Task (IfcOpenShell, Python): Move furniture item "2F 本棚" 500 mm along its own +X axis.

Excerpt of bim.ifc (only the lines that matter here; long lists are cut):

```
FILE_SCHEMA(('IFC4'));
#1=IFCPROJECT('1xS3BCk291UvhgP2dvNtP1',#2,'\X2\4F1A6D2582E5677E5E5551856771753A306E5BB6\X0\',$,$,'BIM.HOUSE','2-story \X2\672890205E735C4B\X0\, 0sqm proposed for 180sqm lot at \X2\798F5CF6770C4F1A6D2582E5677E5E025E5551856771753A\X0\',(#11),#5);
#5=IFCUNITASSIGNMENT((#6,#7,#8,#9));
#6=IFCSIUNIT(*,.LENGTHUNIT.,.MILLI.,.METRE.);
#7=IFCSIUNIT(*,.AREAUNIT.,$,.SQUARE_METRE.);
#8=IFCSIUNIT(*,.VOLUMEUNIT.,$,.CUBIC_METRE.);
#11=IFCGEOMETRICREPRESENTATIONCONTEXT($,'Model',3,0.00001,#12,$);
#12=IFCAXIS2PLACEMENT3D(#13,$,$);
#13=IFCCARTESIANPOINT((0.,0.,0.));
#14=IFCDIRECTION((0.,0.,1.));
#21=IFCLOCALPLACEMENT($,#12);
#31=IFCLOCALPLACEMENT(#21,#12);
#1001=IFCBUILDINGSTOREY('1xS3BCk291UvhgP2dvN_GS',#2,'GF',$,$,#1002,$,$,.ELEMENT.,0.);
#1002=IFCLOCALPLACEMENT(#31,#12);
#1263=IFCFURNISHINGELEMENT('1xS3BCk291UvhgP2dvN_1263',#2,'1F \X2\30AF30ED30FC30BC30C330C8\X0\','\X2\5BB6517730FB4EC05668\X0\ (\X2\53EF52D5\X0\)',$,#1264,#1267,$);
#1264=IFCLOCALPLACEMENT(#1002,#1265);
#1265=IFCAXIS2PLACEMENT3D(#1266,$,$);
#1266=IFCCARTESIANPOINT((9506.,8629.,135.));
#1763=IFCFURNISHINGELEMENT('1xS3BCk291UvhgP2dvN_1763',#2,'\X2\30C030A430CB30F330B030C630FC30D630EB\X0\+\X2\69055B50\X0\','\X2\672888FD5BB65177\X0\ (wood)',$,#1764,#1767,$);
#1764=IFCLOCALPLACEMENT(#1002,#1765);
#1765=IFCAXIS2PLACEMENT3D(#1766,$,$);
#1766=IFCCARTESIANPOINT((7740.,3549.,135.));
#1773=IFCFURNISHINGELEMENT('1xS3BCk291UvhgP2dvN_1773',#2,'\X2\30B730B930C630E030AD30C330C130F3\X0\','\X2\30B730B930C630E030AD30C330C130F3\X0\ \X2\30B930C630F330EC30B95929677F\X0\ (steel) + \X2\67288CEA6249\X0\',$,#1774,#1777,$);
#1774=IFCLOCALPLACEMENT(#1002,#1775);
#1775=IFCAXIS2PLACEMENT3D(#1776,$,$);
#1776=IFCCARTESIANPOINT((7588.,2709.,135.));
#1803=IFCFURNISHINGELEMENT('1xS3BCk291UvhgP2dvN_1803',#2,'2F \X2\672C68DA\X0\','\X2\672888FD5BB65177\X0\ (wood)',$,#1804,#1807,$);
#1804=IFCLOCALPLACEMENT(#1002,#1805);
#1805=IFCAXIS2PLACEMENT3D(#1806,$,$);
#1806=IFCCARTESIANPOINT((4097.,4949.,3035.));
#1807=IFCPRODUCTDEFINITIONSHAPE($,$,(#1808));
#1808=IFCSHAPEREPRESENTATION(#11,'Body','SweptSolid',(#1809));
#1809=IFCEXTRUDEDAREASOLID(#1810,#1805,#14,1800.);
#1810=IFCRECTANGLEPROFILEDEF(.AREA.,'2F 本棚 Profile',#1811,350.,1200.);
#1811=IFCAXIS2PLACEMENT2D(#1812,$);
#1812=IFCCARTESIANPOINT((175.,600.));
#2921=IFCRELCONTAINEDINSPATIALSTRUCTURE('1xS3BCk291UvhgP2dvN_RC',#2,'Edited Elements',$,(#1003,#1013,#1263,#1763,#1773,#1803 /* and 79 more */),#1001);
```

```python
import ifcopenshell
import ifcopenshell.api.geometry
import ifcopenshell.util.placement
import ifcopenshell.util.unit

model = ifcopenshell.open("bim.ifc")
unit_scale = ifcopenshell.util.unit.calculate_unit_scale(model)

item = model.by_guid("1xS3BCk291UvhgP2dvN_1803")
matrix = ifcopenshell.util.placement.get_local_placement(item.ObjectPlacement)
matrix[:3, 3] += matrix[:3, 0] * 0.5 / unit_scale
ifcopenshell.api.geometry.edit_object_placement(model, product=item, matrix=matrix, is_si=False)

print(ifcopenshell.util.placement.get_local_placement(item.ObjectPlacement).round(3) + 0.0)

model.write("bim_updated.ifc")
```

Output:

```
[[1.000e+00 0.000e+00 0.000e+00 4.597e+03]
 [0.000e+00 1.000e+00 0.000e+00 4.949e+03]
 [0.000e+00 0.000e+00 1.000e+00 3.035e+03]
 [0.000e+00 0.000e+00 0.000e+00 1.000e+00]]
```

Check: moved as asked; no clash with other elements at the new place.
